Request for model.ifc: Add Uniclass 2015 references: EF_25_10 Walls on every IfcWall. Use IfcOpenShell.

First a look at what the model holds.

```python
import ifcopenshell

model = ifcopenshell.open("model.ifc")
print(model.schema)
print("classifications:", [c.Name for c in model.by_type("IfcClassification")])
for ifc_class in ("IfcDoor", "IfcRoof", "IfcStair", "IfcWall", "IfcWindow"):
    print(ifc_class, len(model.by_type(ifc_class)))
```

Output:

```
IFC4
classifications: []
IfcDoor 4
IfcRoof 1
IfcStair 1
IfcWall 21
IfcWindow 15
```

```python
import ifcopenshell
import ifcopenshell.api.classification

model = ifcopenshell.open("model.ifc")

system = ifcopenshell.api.classification.add_classification(model, classification="Uniclass 2015")

codes = {
    "IfcWall": ("EF_25_10", "Walls"),
}
for ifc_class, (code, name) in codes.items():
    products = model.by_type(ifc_class)
    ifcopenshell.api.classification.add_reference(
        model, products=products, classification=system, identification=code, name=name
    )
    print(code, len(products))

model.write("model_updated.ifc")
```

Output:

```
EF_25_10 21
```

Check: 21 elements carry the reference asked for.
